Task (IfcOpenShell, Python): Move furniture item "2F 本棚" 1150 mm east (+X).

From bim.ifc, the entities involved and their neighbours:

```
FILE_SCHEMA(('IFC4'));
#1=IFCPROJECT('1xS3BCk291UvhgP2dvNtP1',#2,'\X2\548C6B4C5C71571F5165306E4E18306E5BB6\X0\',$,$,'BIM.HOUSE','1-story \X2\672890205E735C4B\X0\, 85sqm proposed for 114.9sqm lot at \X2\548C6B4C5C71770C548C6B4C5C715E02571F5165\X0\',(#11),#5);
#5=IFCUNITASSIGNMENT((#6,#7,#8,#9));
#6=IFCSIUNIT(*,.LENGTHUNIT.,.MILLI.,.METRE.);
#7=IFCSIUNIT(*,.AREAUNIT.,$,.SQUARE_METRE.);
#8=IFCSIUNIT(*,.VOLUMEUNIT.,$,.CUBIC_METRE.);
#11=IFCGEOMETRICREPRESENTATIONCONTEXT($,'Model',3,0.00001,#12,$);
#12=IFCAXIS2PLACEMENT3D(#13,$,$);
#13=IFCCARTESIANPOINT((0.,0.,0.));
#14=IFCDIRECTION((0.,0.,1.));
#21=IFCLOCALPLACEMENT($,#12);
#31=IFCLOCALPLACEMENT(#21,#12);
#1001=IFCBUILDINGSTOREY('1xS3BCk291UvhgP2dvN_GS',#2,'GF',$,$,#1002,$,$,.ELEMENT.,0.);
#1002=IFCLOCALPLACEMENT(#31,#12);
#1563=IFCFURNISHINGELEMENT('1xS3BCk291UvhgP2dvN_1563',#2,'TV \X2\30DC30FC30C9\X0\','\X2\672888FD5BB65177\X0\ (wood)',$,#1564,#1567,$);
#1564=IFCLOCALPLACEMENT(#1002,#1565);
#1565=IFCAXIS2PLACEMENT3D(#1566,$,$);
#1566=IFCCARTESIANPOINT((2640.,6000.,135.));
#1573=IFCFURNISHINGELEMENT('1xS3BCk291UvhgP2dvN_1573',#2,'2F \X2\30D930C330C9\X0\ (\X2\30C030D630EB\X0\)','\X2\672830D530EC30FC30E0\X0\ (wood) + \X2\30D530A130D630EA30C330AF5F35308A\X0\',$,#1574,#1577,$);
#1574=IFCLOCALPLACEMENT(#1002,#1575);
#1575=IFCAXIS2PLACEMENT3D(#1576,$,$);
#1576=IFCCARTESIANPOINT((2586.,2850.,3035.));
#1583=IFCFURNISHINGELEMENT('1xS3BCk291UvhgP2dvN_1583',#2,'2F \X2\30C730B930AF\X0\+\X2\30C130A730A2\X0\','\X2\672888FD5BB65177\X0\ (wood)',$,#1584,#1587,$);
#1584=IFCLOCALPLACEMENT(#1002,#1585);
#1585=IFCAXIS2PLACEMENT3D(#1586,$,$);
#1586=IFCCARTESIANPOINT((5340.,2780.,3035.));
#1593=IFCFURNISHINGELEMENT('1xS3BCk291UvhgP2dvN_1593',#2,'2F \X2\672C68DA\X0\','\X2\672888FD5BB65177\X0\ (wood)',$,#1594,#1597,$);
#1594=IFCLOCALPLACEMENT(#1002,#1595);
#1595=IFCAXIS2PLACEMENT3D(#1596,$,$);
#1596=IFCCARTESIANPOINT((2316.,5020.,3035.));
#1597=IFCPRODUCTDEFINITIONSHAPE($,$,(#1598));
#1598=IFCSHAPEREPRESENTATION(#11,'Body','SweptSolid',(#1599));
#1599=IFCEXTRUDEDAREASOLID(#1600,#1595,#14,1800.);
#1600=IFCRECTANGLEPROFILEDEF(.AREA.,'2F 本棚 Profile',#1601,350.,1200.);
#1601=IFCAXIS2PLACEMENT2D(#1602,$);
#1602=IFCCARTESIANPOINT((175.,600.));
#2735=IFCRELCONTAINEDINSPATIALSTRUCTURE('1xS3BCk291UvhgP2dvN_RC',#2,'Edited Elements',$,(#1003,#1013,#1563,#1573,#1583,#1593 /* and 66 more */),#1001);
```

```python
import ifcopenshell
import ifcopenshell.api.geometry
import ifcopenshell.util.placement
import ifcopenshell.util.unit

model = ifcopenshell.open("bim.ifc")
unit_scale = ifcopenshell.util.unit.calculate_unit_scale(model)

item = model.by_id(1593)
matrix = ifcopenshell.util.placement.get_local_placement(item.ObjectPlacement)
matrix[0, 3] += 1.15 / unit_scale
ifcopenshell.api.geometry.edit_object_placement(model, product=item, matrix=matrix, is_si=False)

print(ifcopenshell.util.placement.get_local_placement(item.ObjectPlacement).round(3) + 0.0)

model.write("bim-out.ifc")
```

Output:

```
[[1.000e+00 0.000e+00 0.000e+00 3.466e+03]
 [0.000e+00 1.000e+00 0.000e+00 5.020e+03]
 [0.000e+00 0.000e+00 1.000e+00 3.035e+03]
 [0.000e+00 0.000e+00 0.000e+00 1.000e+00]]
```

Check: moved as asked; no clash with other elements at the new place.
